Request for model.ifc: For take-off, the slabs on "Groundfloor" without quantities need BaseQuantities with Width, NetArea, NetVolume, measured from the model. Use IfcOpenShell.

First a look at what the model holds.

```python
import ifcopenshell
import ifcopenshell.util.element
import ifcopenshell.util.unit

model = ifcopenshell.open("model.ifc")
print(model.schema)
for unit_type in ("LENGTHUNIT", "AREAUNIT", "VOLUMEUNIT"):
    print(unit_type, ifcopenshell.util.unit.calculate_unit_scale(model, unit_type))
storey = next(s for s in model.by_type("IfcBuildingStorey") if s.Name == "Groundfloor")
slabs = [e for e in ifcopenshell.util.element.get_decomposition(storey) if e.is_a("IfcSlab")]
for e in sorted(slabs, key=lambda e: e.id()):
    print(e.id(), e.is_a(), e.Name, list(ifcopenshell.util.element.get_psets(e, qtos_only=True)), sep=" | ")
```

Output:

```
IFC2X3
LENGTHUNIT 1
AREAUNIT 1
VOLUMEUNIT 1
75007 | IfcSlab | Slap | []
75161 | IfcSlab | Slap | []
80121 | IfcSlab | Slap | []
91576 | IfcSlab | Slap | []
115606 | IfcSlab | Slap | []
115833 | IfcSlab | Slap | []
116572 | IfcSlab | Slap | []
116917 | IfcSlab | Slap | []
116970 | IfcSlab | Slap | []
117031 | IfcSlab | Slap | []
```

```python
import ifcopenshell
import ifcopenshell.api.pset
import ifcopenshell.geom
import ifcopenshell.util.element
import ifcopenshell.util.shape
import ifcopenshell.util.unit

model = ifcopenshell.open("model.ifc")
unit_scale = ifcopenshell.util.unit.calculate_unit_scale(model)
area_scale = ifcopenshell.util.unit.calculate_unit_scale(model, "AREAUNIT")
volume_scale = ifcopenshell.util.unit.calculate_unit_scale(model, "VOLUMEUNIT")
settings = ifcopenshell.geom.settings()

storey = next(s for s in model.by_type("IfcBuildingStorey") if s.Name == "Groundfloor")
slabs = [e for e in ifcopenshell.util.element.get_decomposition(storey) if e.is_a("IfcSlab")]

for e in sorted(slabs, key=lambda e: e.id()):
    if ifcopenshell.util.element.get_psets(e, qtos_only=True, should_inherit=False):
        continue
    # Geometry comes back in metres, in the element's own axes.
    shape = ifcopenshell.geom.create_shape(settings, e)
    values = {
        "Width": ifcopenshell.util.shape.get_z(shape.geometry) / unit_scale,
        "NetArea": ifcopenshell.util.shape.get_footprint_area(shape.geometry) / area_scale,
        "NetVolume": ifcopenshell.util.shape.get_volume(shape.geometry) / volume_scale,
    }
    qto = ifcopenshell.api.pset.add_qto(model, product=e, name="BaseQuantities")
    ifcopenshell.api.pset.edit_qto(model, qto=qto, properties=values)
    print(e.id(), {k: round(v, 3) for k, v in values.items()})

model.write("model_v2.ifc")
```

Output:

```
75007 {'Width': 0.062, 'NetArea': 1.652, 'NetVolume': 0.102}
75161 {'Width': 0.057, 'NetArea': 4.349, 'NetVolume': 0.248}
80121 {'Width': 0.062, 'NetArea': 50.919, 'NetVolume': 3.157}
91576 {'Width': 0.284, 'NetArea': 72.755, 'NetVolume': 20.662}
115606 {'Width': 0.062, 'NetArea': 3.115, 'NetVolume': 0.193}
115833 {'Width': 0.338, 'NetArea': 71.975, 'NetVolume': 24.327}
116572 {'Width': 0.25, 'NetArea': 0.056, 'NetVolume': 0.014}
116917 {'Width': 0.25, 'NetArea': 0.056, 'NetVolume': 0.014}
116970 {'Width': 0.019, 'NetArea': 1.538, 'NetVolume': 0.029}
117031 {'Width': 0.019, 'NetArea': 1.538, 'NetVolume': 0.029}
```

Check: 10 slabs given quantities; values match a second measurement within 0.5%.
